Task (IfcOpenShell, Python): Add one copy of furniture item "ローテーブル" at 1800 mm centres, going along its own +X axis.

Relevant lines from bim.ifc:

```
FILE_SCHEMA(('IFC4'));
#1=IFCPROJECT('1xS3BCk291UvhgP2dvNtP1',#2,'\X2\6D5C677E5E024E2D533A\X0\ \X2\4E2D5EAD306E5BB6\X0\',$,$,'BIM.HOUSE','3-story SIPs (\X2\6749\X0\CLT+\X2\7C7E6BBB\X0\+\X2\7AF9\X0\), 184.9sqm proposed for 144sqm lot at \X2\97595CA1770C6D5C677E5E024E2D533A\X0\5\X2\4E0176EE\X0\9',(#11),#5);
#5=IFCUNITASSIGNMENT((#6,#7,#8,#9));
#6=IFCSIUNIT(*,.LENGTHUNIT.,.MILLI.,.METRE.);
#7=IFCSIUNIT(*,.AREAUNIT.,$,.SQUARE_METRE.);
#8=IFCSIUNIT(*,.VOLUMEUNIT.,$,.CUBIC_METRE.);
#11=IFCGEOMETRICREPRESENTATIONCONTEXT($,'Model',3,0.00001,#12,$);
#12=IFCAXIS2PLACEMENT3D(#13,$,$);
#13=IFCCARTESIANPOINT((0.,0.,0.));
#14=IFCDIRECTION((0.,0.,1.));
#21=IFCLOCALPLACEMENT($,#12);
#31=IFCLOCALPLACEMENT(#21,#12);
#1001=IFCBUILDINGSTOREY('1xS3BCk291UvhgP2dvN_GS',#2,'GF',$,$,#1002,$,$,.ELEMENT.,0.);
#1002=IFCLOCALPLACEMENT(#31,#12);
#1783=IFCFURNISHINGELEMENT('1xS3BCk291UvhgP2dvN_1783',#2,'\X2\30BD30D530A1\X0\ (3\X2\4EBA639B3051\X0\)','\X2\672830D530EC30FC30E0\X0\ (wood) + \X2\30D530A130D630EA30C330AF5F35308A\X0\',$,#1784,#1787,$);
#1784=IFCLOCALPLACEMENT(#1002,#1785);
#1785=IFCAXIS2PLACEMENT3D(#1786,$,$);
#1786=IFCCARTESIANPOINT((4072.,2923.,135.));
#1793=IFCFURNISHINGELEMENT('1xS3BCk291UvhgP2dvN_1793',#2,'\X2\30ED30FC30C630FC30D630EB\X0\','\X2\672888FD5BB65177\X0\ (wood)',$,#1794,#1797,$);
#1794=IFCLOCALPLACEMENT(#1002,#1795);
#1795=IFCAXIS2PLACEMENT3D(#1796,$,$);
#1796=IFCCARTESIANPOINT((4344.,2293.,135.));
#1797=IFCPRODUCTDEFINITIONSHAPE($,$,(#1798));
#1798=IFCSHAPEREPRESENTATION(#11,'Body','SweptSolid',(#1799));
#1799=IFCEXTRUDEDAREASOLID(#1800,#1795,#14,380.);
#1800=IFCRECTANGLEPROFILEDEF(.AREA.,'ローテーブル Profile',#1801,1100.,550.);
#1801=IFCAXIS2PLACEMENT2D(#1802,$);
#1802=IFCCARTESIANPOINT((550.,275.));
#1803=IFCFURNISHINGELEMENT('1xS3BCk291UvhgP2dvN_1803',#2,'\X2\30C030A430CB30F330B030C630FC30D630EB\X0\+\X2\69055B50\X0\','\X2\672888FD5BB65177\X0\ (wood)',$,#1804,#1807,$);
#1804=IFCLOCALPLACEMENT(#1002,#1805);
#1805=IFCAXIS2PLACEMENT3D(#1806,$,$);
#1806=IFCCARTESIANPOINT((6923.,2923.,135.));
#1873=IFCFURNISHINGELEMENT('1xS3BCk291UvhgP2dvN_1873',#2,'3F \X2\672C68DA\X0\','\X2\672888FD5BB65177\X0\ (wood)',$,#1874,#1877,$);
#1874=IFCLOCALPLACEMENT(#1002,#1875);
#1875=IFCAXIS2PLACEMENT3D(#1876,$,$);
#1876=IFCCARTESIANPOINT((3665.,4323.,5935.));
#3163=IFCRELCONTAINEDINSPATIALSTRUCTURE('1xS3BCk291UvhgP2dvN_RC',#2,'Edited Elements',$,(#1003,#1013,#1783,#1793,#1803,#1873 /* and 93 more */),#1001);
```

```python
import ifcopenshell
import ifcopenshell.api.geometry
import ifcopenshell.api.root
import ifcopenshell.util.element
import ifcopenshell.util.placement

model = ifcopenshell.open("bim.ifc")


def reuse_history(source, copy):
    """copy_class also copies each property set's owner history, people and application; keep the originals."""
    for rel in copy.IsDefinedBy:
        if rel.is_a("IfcRelDefinesByProperties") and (history := rel.RelatingPropertyDefinition.OwnerHistory):
            rel.RelatingPropertyDefinition.OwnerHistory = source.OwnerHistory
            ifcopenshell.util.element.remove_deep2(model, history)


source = model.by_id(1793)
base = ifcopenshell.util.placement.get_local_placement(source.ObjectPlacement)
step = base[:3, 0] * 1800.0

for i in range(1, 2):
    copy = ifcopenshell.api.root.copy_class(model, product=source)
    copy.Representation = ifcopenshell.util.element.copy_deep(
        model, source.Representation, exclude=["IfcGeometricRepresentationContext", "IfcRepresentationMap"]
    )
    reuse_history(source, copy)
    matrix = base.copy()
    matrix[:3, 3] += i * step
    print("added at", matrix[:3, 3].round(3) + 0.0)
    ifcopenshell.api.geometry.edit_object_placement(model, product=copy, matrix=matrix, is_si=False)

model.write("bim-out.ifc")
```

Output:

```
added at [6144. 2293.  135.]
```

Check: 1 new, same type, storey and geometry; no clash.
